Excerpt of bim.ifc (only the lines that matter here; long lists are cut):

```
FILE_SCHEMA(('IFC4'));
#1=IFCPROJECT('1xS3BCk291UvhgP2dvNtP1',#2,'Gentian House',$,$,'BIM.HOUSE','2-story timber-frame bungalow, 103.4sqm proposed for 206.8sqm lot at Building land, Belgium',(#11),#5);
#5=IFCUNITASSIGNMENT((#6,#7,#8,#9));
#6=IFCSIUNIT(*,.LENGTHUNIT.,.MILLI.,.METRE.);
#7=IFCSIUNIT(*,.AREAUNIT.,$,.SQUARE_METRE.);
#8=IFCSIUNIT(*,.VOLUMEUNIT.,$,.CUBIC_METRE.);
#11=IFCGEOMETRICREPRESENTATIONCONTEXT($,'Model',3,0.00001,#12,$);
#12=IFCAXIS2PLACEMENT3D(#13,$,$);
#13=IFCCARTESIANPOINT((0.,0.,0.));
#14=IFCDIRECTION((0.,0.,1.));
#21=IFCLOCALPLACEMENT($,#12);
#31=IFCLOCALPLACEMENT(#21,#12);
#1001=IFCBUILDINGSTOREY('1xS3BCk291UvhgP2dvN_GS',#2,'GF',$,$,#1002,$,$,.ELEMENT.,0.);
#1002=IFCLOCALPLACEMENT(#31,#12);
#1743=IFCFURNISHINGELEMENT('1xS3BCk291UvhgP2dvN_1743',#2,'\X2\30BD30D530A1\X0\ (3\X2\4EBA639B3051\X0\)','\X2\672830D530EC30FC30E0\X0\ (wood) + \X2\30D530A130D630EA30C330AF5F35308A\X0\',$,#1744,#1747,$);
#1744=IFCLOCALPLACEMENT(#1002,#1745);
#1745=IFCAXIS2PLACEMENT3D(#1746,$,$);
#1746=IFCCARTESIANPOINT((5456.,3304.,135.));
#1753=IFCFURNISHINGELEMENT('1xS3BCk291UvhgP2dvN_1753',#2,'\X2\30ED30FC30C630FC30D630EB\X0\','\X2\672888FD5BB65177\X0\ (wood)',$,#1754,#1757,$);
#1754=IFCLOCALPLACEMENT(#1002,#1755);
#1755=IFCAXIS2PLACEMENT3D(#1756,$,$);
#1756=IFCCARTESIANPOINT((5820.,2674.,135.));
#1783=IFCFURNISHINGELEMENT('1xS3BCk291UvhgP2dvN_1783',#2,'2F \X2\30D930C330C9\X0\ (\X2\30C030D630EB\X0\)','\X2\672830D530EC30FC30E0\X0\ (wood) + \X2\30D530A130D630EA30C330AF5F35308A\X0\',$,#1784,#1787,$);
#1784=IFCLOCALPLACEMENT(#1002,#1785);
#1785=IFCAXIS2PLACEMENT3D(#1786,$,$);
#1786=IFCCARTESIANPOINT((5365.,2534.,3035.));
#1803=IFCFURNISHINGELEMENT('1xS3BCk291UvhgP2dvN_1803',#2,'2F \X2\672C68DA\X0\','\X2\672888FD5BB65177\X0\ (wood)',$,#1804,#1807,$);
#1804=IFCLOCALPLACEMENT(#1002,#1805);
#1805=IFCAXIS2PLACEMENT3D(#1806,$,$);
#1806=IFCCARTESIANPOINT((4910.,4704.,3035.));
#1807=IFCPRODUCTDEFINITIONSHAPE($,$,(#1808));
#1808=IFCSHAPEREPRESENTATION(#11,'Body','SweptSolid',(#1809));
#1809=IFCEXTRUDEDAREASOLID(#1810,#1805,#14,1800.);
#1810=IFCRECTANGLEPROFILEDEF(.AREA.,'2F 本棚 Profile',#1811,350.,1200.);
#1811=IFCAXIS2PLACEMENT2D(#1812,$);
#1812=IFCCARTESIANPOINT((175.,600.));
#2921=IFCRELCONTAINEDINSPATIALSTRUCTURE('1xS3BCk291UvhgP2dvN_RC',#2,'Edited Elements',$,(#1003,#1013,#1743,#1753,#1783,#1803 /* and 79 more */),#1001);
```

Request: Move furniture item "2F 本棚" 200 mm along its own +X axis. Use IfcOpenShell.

```python
import ifcopenshell
import ifcopenshell.api.geometry
import ifcopenshell.util.placement

model = ifcopenshell.open("bim.ifc")

item = model.by_id(1803)
matrix = ifcopenshell.util.placement.get_local_placement(item.ObjectPlacement)
matrix[:3, 3] += matrix[:3, 0] * 200.0
ifcopenshell.api.geometry.edit_object_placement(model, product=item, matrix=matrix, is_si=False)

print(ifcopenshell.util.placement.get_local_placement(item.ObjectPlacement).round(3) + 0.0)

model.write("bim_edited.ifc")
```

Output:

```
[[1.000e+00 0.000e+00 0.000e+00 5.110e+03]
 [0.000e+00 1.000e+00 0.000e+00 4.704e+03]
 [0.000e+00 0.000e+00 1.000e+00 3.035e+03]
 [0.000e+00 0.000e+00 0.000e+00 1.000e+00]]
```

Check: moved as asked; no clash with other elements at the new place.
